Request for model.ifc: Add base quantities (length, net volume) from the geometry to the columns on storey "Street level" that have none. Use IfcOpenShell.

First a look at what the model holds.

```python
import ifcopenshell
import ifcopenshell.util.element
import ifcopenshell.util.unit

model = ifcopenshell.open("model.ifc")
print(model.schema)
for unit_type in ("LENGTHUNIT", "AREAUNIT", "VOLUMEUNIT"):
    print(unit_type, ifcopenshell.util.unit.calculate_unit_scale(model, unit_type))
storey = next(s for s in model.by_type("IfcBuildingStorey") if s.Name == "Street level")
columns = [e for e in ifcopenshell.util.element.get_decomposition(storey) if e.is_a("IfcColumn")]
for e in sorted(columns, key=lambda e: e.id()):
    print(e.id(), e.is_a(), e.Name, list(ifcopenshell.util.element.get_psets(e, qtos_only=True)), sep=" | ")
```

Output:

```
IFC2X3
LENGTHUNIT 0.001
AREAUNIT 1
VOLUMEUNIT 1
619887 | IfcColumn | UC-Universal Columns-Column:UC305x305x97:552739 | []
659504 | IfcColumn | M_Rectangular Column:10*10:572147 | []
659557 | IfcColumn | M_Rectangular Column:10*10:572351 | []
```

```python
import ifcopenshell
import ifcopenshell.api.pset
import ifcopenshell.geom
import ifcopenshell.util.element
import ifcopenshell.util.shape
import ifcopenshell.util.unit

model = ifcopenshell.open("model.ifc")
unit_scale = ifcopenshell.util.unit.calculate_unit_scale(model)
volume_scale = ifcopenshell.util.unit.calculate_unit_scale(model, "VOLUMEUNIT")
settings = ifcopenshell.geom.settings()

storey = next(s for s in model.by_type("IfcBuildingStorey") if s.Name == "Street level")
columns = [e for e in ifcopenshell.util.element.get_decomposition(storey) if e.is_a("IfcColumn")]

for e in sorted(columns, key=lambda e: e.id()):
    if ifcopenshell.util.element.get_psets(e, qtos_only=True, should_inherit=False):
        continue
    # Geometry comes back in metres, in the element's own axes.
    shape = ifcopenshell.geom.create_shape(settings, e)
    values = {
        "Length": ifcopenshell.util.shape.get_z(shape.geometry) / unit_scale,
        "NetVolume": ifcopenshell.util.shape.get_volume(shape.geometry) / volume_scale,
    }
    qto = ifcopenshell.api.pset.add_qto(model, product=e, name="BaseQuantities")
    ifcopenshell.api.pset.edit_qto(model, qto=qto, properties=values)
    print(e.id(), {k: round(v, 3) for k, v in values.items()})

model.write("model_edited.ifc")
```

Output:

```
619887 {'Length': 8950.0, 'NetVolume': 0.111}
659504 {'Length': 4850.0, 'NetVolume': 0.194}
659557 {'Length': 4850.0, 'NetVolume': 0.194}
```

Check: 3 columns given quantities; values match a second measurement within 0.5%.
